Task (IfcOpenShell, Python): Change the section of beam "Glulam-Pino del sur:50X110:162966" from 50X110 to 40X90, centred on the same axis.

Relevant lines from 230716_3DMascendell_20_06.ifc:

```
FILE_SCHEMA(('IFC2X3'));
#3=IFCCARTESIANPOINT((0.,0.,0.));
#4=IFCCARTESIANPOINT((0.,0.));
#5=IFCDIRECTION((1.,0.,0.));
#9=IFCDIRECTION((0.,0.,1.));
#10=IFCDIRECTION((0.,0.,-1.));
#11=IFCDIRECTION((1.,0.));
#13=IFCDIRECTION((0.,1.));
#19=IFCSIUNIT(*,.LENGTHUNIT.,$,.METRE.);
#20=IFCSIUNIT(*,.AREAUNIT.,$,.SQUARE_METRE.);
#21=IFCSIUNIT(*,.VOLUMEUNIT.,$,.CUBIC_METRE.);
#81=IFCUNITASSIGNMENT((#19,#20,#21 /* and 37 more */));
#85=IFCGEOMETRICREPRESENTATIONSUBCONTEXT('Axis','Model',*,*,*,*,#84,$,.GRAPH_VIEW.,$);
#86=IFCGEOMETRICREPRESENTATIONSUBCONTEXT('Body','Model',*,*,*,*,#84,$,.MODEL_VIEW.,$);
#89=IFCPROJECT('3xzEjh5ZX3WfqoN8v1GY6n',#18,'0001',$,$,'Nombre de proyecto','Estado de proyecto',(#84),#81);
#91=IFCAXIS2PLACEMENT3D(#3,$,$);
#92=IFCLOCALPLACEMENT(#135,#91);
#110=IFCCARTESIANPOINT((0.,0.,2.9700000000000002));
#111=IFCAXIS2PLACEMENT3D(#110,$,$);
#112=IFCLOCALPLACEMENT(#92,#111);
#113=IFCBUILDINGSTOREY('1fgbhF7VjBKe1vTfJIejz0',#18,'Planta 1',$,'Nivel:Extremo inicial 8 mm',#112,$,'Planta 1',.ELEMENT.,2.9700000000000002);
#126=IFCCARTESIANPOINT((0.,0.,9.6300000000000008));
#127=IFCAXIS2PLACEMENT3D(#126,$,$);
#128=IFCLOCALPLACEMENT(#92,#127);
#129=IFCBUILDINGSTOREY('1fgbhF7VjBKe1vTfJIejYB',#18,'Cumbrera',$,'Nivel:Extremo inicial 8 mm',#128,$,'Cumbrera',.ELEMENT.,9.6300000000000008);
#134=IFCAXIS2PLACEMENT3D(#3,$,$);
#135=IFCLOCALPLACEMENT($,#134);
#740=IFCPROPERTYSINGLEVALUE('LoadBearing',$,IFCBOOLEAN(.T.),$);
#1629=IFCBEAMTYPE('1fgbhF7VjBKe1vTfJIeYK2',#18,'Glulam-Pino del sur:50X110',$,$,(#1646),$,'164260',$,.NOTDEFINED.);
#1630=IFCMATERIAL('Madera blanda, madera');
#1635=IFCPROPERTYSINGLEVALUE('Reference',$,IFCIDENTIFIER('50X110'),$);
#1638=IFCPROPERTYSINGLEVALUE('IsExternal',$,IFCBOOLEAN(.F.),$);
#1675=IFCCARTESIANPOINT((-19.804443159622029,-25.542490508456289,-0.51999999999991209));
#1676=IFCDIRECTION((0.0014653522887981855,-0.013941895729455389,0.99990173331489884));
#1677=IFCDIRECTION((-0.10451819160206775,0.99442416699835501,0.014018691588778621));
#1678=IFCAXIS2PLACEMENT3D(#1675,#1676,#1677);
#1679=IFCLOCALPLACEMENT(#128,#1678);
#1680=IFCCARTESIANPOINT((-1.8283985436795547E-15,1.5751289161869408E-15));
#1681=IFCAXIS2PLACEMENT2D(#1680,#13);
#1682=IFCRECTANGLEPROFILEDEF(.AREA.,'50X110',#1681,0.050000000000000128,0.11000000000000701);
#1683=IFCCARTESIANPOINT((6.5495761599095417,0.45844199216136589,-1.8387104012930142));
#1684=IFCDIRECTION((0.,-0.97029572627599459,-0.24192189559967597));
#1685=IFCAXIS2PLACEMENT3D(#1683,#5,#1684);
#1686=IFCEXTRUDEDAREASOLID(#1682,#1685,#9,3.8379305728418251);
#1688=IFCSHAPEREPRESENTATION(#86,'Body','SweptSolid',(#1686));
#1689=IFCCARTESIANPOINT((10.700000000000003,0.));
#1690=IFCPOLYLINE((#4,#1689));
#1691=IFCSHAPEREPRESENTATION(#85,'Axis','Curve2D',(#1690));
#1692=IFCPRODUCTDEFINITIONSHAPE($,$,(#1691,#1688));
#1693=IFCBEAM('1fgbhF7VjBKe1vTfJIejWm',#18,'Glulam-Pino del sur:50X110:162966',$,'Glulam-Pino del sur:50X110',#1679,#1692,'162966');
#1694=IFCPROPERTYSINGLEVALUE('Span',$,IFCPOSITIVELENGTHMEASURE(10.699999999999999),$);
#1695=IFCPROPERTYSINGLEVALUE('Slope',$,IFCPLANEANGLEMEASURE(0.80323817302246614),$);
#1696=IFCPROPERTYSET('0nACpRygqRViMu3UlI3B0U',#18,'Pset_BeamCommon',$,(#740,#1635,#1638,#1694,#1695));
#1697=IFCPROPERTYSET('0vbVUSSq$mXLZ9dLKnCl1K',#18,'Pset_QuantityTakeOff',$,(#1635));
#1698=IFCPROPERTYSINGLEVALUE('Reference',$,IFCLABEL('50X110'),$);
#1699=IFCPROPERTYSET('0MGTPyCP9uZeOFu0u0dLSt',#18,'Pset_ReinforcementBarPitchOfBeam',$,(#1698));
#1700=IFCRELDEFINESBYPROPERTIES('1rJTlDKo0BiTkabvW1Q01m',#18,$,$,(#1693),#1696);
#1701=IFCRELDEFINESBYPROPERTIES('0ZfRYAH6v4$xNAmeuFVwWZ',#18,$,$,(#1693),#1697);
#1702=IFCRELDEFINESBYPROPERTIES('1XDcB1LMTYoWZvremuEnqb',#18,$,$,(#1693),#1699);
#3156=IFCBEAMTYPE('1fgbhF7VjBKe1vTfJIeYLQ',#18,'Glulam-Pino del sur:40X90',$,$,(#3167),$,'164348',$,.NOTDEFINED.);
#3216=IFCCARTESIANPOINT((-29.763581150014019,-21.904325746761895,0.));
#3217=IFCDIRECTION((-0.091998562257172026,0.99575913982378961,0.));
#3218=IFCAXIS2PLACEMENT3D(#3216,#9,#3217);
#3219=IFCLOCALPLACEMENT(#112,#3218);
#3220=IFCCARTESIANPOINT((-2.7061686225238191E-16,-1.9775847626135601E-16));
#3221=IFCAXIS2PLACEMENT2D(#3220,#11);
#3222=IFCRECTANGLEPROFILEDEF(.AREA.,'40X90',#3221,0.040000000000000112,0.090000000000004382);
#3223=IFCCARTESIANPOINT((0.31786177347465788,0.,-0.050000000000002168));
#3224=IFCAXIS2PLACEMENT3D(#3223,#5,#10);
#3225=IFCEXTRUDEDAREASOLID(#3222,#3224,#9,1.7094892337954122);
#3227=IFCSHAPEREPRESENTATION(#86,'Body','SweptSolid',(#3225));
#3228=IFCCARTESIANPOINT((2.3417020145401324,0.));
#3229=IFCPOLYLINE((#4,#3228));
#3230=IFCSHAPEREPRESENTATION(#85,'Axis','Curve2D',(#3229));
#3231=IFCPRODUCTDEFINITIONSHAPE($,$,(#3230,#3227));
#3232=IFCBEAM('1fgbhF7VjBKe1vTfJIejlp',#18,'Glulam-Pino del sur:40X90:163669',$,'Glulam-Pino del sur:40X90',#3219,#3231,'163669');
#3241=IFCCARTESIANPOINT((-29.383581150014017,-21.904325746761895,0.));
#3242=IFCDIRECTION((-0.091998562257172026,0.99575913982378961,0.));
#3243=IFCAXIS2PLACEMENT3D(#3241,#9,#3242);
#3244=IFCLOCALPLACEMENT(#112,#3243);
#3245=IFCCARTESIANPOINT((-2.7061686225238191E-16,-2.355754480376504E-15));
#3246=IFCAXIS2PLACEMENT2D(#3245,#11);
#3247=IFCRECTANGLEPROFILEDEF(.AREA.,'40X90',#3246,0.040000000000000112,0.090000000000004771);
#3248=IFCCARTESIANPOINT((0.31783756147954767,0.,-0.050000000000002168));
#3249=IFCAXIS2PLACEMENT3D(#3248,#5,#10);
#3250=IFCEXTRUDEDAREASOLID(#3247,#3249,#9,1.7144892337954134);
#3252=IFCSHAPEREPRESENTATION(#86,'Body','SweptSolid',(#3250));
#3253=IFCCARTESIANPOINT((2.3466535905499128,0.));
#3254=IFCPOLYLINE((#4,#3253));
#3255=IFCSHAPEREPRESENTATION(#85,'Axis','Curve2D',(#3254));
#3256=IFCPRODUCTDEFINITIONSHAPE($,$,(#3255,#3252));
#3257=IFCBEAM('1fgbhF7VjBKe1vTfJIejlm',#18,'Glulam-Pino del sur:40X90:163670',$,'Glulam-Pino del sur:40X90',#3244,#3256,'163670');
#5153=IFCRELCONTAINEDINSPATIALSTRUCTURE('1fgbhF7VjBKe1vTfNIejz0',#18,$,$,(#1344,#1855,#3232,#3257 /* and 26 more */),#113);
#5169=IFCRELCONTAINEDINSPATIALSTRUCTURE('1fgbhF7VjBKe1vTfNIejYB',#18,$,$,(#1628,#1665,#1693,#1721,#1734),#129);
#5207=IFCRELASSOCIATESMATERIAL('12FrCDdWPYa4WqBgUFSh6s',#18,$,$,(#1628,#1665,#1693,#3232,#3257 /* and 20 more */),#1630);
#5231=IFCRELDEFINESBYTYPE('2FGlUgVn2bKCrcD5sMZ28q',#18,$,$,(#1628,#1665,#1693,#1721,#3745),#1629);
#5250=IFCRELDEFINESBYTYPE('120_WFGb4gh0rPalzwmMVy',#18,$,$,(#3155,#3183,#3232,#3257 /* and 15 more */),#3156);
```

```python
import ifcopenshell
import ifcopenshell.api.pset
import ifcopenshell.api.type
import ifcopenshell.util.element
import ifcopenshell.util.representation

model = ifcopenshell.open("230716_3DMascendell_20_06.ifc")

member = model.by_guid("1fgbhF7VjBKe1vTfJIejWm")
source = next(p for p in model.by_type("IfcRectangleProfileDef") if p.ProfileName == "40X90")

body = ifcopenshell.util.representation.get_representation(member, "Model", "Body")
solid = body.Items[0]
old_profile = solid.SweptArea

# Copy the section's sizes but keep this member's own profile position.
profile = ifcopenshell.util.element.copy(model, source)
profile.Position = old_profile.Position
solid.SweptArea = profile
if not model.get_total_inverses(old_profile):
    ifcopenshell.util.element.remove_deep2(model, old_profile)

new_type = model.by_id(3156)
ifcopenshell.api.type.assign_type(
    model, related_objects=[member], relating_type=new_type, should_map_representations=False
)
member.Name = member.Name.replace("50X110", "40X90")
member.ObjectType = "Glulam-Pino del sur:40X90"
pset = model.by_id(ifcopenshell.util.element.get_pset(member, "Pset_BeamCommon", should_inherit=False)["id"])
ifcopenshell.api.pset.edit_pset(model, pset=pset, properties={"Reference": "40X90"})
pset = model.by_id(ifcopenshell.util.element.get_pset(member, "Pset_QuantityTakeOff", should_inherit=False)["id"])
ifcopenshell.api.pset.edit_pset(model, pset=pset, properties={"Reference": "40X90"})
pset = model.by_id(ifcopenshell.util.element.get_pset(member, "Pset_ReinforcementBarPitchOfBeam", should_inherit=False)["id"])
ifcopenshell.api.pset.edit_pset(model, pset=pset, properties={"Reference": "40X90"})

print(solid.SweptArea)

model.write("230716_3DMascendell_20_06-out.ifc")
```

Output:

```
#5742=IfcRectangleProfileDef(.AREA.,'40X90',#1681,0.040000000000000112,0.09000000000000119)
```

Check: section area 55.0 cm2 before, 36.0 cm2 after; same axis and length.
